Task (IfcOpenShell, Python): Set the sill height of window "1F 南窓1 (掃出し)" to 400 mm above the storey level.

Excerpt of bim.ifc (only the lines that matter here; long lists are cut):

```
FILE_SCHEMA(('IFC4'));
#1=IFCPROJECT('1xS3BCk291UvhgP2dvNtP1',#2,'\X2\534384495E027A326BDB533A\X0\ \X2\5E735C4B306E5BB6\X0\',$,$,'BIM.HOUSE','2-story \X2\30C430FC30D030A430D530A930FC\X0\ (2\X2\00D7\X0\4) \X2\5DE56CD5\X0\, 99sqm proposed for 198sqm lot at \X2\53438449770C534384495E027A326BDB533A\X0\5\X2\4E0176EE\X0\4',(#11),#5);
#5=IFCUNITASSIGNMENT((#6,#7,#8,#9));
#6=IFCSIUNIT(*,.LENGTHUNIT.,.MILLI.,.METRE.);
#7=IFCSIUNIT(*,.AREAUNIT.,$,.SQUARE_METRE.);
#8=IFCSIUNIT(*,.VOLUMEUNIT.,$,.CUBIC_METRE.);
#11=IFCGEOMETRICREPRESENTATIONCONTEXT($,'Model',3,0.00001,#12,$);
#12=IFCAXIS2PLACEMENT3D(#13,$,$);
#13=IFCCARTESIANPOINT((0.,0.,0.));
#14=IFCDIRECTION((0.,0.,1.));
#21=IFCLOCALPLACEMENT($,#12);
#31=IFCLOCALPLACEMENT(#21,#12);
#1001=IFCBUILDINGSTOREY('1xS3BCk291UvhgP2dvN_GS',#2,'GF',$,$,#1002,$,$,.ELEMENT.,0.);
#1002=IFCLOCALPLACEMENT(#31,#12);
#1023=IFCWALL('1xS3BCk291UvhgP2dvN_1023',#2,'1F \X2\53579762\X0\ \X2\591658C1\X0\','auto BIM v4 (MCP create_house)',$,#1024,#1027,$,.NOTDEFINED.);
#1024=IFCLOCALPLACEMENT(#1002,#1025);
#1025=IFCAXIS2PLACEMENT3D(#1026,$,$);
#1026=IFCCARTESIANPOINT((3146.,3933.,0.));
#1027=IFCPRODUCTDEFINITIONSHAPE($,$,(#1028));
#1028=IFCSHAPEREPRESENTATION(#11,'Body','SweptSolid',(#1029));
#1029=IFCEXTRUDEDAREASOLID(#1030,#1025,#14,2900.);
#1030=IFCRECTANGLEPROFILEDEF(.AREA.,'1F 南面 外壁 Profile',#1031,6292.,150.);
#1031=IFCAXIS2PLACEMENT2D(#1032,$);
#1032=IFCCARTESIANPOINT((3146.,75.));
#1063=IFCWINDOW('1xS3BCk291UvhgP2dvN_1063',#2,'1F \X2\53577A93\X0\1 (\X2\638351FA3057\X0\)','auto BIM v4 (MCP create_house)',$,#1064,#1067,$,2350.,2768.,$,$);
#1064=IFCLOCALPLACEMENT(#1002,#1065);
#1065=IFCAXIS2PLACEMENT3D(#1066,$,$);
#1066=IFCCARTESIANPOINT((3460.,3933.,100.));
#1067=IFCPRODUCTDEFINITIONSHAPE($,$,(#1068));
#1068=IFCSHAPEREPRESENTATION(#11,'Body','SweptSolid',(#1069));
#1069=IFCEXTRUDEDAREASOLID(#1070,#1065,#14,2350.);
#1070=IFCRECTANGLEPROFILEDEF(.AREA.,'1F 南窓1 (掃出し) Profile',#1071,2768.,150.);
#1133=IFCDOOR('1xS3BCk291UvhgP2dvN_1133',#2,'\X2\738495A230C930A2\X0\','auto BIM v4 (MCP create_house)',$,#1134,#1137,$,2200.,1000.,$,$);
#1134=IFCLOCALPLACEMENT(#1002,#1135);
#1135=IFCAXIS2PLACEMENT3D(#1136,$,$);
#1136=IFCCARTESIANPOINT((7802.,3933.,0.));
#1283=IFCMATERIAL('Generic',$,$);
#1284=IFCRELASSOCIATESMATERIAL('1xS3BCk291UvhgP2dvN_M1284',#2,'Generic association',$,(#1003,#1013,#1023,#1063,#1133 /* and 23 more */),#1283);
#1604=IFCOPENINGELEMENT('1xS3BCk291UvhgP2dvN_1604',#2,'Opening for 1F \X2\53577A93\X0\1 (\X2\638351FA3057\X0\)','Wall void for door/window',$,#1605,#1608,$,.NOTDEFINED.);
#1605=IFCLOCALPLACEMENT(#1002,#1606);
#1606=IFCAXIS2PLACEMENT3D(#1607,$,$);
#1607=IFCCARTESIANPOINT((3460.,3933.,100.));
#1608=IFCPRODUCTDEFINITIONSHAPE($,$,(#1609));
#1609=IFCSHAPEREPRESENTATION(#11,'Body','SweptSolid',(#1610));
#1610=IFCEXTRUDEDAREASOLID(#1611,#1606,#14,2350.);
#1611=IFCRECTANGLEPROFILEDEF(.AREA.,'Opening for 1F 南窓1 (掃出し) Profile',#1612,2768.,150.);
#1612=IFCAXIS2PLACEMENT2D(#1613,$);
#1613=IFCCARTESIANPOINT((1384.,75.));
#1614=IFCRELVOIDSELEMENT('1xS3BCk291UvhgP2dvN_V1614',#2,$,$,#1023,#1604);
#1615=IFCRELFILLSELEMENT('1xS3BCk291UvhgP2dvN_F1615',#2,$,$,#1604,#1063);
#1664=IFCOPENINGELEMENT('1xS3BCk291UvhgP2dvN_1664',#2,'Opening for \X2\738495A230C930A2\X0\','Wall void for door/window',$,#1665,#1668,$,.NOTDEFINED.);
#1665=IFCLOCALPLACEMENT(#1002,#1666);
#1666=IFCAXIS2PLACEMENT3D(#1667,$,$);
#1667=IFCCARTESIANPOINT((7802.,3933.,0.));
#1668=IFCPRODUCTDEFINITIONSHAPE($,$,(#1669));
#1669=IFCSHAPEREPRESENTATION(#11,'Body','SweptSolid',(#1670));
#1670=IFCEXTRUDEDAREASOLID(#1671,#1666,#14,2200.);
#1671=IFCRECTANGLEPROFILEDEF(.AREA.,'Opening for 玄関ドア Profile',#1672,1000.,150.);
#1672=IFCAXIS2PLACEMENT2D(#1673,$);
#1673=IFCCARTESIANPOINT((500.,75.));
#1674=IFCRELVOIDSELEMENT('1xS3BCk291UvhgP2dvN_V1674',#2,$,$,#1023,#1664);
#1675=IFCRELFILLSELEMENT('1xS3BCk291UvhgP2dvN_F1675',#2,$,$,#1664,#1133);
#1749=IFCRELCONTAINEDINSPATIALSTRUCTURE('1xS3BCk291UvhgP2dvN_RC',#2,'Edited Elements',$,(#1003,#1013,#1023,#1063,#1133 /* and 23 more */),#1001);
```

```python
import numpy as np
import ifcopenshell
import ifcopenshell.api.geometry
import ifcopenshell.geom
import ifcopenshell.util.element
import ifcopenshell.util.placement
import ifcopenshell.util.shape
import ifcopenshell.util.unit

model = ifcopenshell.open("bim.ifc")
unit_scale = ifcopenshell.util.unit.calculate_unit_scale(model)

window = model.by_guid("1xS3BCk291UvhgP2dvN_1063")
opening = window.FillsVoids[0].RelatingOpeningElement
storey = ifcopenshell.util.element.get_container(window, ifc_class="IfcBuildingStorey")
level = ifcopenshell.util.placement.get_local_placement(storey.ObjectPlacement)[2, 3]

# The opening's origin need not be at the sill, so measure its lowest point.
shape = ifcopenshell.geom.create_shape(ifcopenshell.geom.settings(), opening)
bottom = ifcopenshell.util.shape.get_shape_bottom_elevation(shape, shape.geometry) / unit_scale
dz = level + 400.0 - bottom

shift = np.array([0.0, 0.0, dz])
# The window is not placed relative to its opening, so move both.
for product in (opening, window):
    matrix = ifcopenshell.util.placement.get_local_placement(product.ObjectPlacement)
    matrix[:3, 3] += shift
    ifcopenshell.api.geometry.edit_object_placement(model, product=product, matrix=matrix, is_si=False)

print(f"moved by {dz * unit_scale:+.3f} m")

model.write("bim_updated.ifc")
```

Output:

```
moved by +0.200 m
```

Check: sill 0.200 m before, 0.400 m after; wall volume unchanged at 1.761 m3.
